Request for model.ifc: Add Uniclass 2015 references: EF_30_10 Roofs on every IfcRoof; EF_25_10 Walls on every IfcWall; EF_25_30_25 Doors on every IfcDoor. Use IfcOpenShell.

First a look at what the model holds.

```python
import ifcopenshell

model = ifcopenshell.open("model.ifc")
print(model.schema)
print("classifications:", [c.Name for c in model.by_type("IfcClassification")])
for ifc_class in ("IfcDoor", "IfcRoof", "IfcStair", "IfcWall", "IfcWindow"):
    print(ifc_class, len(model.by_type(ifc_class)))
```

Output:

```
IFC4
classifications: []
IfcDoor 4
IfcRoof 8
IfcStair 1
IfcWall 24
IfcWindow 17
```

```python
import ifcopenshell
import ifcopenshell.api.classification

model = ifcopenshell.open("model.ifc")

system = ifcopenshell.api.classification.add_classification(model, classification="Uniclass 2015")

codes = {
    "IfcRoof": ("EF_30_10", "Roofs"),
    "IfcWall": ("EF_25_10", "Walls"),
    "IfcDoor": ("EF_25_30_25", "Doors"),
}
for ifc_class, (code, name) in codes.items():
    products = model.by_type(ifc_class)
    ifcopenshell.api.classification.add_reference(
        model, products=products, classification=system, identification=code, name=name
    )
    print(code, len(products))

model.write("model_v2.ifc")
```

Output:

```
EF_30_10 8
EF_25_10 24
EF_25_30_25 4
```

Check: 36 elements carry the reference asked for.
